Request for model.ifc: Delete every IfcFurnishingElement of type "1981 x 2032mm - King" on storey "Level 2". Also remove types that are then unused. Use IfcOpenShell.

First a look at what the model holds.

```python
import ifcopenshell
import ifcopenshell.util.element

model = ifcopenshell.open("model.ifc")
print(model.schema)
storey = next(s for s in model.by_type("IfcBuildingStorey") if s.Name == "Level 2")
furniture = [e for e in ifcopenshell.util.element.get_decomposition(storey) if e.is_a("IfcFurnishingElement")]
seen = {}
for e in furniture:
    element_type = ifcopenshell.util.element.get_type(e)
    name = element_type.Name if element_type not in (None, e) else None
    seen[name] = seen.get(name, 0) + 1
for name, count in sorted(seen.items(), key=str):
    print(count, "x", name)
```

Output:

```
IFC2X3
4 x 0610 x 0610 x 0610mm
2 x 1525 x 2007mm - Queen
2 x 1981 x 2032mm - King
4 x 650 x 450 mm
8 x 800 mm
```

```python
import ifcopenshell
import ifcopenshell.api.root
import ifcopenshell.util.element

model = ifcopenshell.open("model.ifc")

storey = next(s for s in model.by_type("IfcBuildingStorey") if s.Name == "Level 2")
furniture = [e for e in ifcopenshell.util.element.get_decomposition(storey) if e.is_a("IfcFurnishingElement")]
targets = [e for e in furniture if (t := ifcopenshell.util.element.get_type(e)) not in (None, e) and t.Name == "1981 x 2032mm - King"]
types = {ifcopenshell.util.element.get_type(e) for e in targets} - {None, *targets}

for e in targets:
    ifcopenshell.api.root.remove_product(model, product=e)
print(len(targets), "removed")

unused = [t for t in types if not ifcopenshell.util.element.get_types(t)]
for t in unused:
    ifcopenshell.api.root.remove_product(model, product=t)
print(len(unused), "unused types removed")

model.write("model-out.ifc")
```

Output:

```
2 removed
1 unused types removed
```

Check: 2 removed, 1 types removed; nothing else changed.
